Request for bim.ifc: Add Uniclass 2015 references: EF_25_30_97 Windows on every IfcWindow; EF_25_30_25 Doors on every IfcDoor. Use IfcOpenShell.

First a look at what the model holds.

```python
import ifcopenshell

model = ifcopenshell.open("bim.ifc")
print(model.schema)
print("classifications:", [c.Name for c in model.by_type("IfcClassification")])
for ifc_class in ("IfcDoor", "IfcRoof", "IfcStair", "IfcWall", "IfcWindow"):
    print(ifc_class, len(model.by_type(ifc_class)))
```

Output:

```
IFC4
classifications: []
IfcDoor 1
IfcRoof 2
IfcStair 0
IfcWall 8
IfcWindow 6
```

```python
import ifcopenshell
import ifcopenshell.api.classification

model = ifcopenshell.open("bim.ifc")

system = ifcopenshell.api.classification.add_classification(model, classification="Uniclass 2015")

codes = {
    "IfcWindow": ("EF_25_30_97", "Windows"),
    "IfcDoor": ("EF_25_30_25", "Doors"),
}
for ifc_class, (code, name) in codes.items():
    products = model.by_type(ifc_class)
    ifcopenshell.api.classification.add_reference(
        model, products=products, classification=system, identification=code, name=name
    )
    print(code, len(products))

model.write("bim-out.ifc")
```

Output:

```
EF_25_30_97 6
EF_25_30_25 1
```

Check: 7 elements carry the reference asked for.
